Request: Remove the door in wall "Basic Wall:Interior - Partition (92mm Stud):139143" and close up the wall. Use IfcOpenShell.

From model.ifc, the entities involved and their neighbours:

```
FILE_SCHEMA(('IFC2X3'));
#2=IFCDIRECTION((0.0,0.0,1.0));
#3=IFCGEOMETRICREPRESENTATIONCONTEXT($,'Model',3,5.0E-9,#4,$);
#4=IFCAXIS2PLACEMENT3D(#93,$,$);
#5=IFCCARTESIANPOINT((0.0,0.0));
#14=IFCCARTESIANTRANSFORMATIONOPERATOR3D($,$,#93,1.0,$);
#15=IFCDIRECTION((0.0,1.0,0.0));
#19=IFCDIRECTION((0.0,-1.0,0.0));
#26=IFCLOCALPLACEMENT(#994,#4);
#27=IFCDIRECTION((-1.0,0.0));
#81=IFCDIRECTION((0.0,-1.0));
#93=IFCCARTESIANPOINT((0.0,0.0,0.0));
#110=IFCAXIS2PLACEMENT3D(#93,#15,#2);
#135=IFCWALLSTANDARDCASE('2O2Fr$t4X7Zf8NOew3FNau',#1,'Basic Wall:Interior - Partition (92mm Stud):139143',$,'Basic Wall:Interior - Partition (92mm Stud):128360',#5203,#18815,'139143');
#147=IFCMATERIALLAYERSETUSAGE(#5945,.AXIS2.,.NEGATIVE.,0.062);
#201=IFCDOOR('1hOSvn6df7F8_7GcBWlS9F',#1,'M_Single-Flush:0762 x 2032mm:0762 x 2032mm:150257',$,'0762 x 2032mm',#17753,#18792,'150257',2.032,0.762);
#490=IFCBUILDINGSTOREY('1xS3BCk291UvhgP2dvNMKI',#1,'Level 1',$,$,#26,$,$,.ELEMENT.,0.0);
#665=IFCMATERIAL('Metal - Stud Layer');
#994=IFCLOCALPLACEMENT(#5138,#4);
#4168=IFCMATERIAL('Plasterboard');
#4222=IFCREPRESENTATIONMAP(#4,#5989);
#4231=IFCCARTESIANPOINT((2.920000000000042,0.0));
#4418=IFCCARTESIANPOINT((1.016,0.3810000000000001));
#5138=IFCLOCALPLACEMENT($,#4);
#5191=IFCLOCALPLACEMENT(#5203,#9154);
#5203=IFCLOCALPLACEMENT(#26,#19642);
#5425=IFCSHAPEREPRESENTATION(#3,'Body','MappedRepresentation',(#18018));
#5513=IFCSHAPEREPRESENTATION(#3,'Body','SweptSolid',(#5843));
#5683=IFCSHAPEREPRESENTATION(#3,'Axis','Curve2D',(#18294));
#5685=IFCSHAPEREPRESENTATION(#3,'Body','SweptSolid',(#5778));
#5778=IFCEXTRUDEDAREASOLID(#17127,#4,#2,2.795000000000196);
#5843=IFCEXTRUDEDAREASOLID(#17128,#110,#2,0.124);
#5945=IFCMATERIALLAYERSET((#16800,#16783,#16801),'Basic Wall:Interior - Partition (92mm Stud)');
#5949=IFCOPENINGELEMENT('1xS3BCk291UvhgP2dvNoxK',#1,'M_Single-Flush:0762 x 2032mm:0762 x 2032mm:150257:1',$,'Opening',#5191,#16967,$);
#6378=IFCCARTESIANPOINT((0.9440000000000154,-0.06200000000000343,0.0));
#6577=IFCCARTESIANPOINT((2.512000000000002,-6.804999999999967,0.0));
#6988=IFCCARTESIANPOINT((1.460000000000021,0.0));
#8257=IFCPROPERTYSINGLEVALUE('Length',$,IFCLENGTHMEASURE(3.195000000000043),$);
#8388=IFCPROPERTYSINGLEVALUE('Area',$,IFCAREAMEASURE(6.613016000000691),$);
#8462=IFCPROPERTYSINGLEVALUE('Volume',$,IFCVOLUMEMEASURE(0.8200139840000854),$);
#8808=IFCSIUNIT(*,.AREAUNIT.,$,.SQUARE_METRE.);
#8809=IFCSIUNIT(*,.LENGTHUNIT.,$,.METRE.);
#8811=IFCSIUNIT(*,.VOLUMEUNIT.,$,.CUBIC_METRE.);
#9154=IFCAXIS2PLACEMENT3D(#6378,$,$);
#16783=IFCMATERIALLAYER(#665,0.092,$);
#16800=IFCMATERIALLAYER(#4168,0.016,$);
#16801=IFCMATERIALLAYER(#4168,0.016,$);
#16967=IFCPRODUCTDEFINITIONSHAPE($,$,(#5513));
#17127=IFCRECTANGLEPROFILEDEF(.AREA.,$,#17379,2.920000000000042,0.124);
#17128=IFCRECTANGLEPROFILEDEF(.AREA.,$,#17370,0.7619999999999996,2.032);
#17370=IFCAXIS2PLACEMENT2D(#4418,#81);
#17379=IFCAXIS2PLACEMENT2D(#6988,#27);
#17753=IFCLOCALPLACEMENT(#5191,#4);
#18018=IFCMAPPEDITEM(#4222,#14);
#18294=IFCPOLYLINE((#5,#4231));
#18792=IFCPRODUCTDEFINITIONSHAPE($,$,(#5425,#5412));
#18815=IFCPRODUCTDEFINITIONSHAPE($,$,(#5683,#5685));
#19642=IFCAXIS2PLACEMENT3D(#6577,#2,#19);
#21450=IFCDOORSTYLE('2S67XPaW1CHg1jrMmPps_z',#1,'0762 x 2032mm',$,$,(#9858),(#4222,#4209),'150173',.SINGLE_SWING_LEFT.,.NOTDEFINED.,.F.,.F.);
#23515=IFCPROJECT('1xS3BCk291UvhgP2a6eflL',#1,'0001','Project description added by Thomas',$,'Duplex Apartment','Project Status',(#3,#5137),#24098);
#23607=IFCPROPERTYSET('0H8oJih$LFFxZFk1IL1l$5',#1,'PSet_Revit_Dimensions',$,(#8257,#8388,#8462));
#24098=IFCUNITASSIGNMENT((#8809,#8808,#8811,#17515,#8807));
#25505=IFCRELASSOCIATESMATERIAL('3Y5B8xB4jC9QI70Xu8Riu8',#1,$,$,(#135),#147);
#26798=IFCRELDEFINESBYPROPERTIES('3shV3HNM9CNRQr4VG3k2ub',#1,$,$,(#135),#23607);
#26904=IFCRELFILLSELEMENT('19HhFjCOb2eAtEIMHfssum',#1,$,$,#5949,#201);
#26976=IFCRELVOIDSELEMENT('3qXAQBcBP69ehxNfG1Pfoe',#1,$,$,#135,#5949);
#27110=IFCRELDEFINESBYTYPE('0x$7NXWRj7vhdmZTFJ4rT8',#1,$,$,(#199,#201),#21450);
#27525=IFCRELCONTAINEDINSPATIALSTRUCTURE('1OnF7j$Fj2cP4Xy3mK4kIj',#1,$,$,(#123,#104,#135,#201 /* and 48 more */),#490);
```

```python
import ifcopenshell
import ifcopenshell.api.feature
import ifcopenshell.api.pset
import ifcopenshell.api.root
import ifcopenshell.geom
import ifcopenshell.util.element
import ifcopenshell.util.shape
import ifcopenshell.util.unit

model = ifcopenshell.open("model.ifc")
area_scale = ifcopenshell.util.unit.calculate_unit_scale(model, "AREAUNIT")
volume_scale = ifcopenshell.util.unit.calculate_unit_scale(model, "VOLUMEUNIT")
settings = ifcopenshell.geom.settings()


def volume(element):
    """Net volume in cubic metres, openings subtracted."""
    shape = ifcopenshell.geom.create_shape(settings, element)
    return ifcopenshell.util.shape.get_volume(shape.geometry)


door = model.by_id(201)
opening = door.FillsVoids[0].RelatingOpeningElement
wall = opening.VoidsElements[0].RelatingBuildingElement
before = volume(wall)

ifcopenshell.api.root.remove_product(model, product=door)
ifcopenshell.api.feature.remove_feature(model, feature=opening)

after = volume(wall)
thickness = 0.124  # wall thickness in metres

# Update the wall's stored quantities.
pset = model.by_id(ifcopenshell.util.element.get_pset(wall, "PSet_Revit_Dimensions", should_inherit=False)["id"])
ifcopenshell.api.pset.edit_pset(model, pset=pset, properties={
    "Area": model.create_entity("IfcAreaMeasure", after / thickness / area_scale),
    "Volume": model.create_entity("IfcVolumeMeasure", after / volume_scale),
})

print(f"wall volume {before:.3f} -> {after:.3f} m3")

model.write("model_edited.ifc")
```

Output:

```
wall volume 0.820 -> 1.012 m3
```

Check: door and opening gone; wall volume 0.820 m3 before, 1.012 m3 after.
